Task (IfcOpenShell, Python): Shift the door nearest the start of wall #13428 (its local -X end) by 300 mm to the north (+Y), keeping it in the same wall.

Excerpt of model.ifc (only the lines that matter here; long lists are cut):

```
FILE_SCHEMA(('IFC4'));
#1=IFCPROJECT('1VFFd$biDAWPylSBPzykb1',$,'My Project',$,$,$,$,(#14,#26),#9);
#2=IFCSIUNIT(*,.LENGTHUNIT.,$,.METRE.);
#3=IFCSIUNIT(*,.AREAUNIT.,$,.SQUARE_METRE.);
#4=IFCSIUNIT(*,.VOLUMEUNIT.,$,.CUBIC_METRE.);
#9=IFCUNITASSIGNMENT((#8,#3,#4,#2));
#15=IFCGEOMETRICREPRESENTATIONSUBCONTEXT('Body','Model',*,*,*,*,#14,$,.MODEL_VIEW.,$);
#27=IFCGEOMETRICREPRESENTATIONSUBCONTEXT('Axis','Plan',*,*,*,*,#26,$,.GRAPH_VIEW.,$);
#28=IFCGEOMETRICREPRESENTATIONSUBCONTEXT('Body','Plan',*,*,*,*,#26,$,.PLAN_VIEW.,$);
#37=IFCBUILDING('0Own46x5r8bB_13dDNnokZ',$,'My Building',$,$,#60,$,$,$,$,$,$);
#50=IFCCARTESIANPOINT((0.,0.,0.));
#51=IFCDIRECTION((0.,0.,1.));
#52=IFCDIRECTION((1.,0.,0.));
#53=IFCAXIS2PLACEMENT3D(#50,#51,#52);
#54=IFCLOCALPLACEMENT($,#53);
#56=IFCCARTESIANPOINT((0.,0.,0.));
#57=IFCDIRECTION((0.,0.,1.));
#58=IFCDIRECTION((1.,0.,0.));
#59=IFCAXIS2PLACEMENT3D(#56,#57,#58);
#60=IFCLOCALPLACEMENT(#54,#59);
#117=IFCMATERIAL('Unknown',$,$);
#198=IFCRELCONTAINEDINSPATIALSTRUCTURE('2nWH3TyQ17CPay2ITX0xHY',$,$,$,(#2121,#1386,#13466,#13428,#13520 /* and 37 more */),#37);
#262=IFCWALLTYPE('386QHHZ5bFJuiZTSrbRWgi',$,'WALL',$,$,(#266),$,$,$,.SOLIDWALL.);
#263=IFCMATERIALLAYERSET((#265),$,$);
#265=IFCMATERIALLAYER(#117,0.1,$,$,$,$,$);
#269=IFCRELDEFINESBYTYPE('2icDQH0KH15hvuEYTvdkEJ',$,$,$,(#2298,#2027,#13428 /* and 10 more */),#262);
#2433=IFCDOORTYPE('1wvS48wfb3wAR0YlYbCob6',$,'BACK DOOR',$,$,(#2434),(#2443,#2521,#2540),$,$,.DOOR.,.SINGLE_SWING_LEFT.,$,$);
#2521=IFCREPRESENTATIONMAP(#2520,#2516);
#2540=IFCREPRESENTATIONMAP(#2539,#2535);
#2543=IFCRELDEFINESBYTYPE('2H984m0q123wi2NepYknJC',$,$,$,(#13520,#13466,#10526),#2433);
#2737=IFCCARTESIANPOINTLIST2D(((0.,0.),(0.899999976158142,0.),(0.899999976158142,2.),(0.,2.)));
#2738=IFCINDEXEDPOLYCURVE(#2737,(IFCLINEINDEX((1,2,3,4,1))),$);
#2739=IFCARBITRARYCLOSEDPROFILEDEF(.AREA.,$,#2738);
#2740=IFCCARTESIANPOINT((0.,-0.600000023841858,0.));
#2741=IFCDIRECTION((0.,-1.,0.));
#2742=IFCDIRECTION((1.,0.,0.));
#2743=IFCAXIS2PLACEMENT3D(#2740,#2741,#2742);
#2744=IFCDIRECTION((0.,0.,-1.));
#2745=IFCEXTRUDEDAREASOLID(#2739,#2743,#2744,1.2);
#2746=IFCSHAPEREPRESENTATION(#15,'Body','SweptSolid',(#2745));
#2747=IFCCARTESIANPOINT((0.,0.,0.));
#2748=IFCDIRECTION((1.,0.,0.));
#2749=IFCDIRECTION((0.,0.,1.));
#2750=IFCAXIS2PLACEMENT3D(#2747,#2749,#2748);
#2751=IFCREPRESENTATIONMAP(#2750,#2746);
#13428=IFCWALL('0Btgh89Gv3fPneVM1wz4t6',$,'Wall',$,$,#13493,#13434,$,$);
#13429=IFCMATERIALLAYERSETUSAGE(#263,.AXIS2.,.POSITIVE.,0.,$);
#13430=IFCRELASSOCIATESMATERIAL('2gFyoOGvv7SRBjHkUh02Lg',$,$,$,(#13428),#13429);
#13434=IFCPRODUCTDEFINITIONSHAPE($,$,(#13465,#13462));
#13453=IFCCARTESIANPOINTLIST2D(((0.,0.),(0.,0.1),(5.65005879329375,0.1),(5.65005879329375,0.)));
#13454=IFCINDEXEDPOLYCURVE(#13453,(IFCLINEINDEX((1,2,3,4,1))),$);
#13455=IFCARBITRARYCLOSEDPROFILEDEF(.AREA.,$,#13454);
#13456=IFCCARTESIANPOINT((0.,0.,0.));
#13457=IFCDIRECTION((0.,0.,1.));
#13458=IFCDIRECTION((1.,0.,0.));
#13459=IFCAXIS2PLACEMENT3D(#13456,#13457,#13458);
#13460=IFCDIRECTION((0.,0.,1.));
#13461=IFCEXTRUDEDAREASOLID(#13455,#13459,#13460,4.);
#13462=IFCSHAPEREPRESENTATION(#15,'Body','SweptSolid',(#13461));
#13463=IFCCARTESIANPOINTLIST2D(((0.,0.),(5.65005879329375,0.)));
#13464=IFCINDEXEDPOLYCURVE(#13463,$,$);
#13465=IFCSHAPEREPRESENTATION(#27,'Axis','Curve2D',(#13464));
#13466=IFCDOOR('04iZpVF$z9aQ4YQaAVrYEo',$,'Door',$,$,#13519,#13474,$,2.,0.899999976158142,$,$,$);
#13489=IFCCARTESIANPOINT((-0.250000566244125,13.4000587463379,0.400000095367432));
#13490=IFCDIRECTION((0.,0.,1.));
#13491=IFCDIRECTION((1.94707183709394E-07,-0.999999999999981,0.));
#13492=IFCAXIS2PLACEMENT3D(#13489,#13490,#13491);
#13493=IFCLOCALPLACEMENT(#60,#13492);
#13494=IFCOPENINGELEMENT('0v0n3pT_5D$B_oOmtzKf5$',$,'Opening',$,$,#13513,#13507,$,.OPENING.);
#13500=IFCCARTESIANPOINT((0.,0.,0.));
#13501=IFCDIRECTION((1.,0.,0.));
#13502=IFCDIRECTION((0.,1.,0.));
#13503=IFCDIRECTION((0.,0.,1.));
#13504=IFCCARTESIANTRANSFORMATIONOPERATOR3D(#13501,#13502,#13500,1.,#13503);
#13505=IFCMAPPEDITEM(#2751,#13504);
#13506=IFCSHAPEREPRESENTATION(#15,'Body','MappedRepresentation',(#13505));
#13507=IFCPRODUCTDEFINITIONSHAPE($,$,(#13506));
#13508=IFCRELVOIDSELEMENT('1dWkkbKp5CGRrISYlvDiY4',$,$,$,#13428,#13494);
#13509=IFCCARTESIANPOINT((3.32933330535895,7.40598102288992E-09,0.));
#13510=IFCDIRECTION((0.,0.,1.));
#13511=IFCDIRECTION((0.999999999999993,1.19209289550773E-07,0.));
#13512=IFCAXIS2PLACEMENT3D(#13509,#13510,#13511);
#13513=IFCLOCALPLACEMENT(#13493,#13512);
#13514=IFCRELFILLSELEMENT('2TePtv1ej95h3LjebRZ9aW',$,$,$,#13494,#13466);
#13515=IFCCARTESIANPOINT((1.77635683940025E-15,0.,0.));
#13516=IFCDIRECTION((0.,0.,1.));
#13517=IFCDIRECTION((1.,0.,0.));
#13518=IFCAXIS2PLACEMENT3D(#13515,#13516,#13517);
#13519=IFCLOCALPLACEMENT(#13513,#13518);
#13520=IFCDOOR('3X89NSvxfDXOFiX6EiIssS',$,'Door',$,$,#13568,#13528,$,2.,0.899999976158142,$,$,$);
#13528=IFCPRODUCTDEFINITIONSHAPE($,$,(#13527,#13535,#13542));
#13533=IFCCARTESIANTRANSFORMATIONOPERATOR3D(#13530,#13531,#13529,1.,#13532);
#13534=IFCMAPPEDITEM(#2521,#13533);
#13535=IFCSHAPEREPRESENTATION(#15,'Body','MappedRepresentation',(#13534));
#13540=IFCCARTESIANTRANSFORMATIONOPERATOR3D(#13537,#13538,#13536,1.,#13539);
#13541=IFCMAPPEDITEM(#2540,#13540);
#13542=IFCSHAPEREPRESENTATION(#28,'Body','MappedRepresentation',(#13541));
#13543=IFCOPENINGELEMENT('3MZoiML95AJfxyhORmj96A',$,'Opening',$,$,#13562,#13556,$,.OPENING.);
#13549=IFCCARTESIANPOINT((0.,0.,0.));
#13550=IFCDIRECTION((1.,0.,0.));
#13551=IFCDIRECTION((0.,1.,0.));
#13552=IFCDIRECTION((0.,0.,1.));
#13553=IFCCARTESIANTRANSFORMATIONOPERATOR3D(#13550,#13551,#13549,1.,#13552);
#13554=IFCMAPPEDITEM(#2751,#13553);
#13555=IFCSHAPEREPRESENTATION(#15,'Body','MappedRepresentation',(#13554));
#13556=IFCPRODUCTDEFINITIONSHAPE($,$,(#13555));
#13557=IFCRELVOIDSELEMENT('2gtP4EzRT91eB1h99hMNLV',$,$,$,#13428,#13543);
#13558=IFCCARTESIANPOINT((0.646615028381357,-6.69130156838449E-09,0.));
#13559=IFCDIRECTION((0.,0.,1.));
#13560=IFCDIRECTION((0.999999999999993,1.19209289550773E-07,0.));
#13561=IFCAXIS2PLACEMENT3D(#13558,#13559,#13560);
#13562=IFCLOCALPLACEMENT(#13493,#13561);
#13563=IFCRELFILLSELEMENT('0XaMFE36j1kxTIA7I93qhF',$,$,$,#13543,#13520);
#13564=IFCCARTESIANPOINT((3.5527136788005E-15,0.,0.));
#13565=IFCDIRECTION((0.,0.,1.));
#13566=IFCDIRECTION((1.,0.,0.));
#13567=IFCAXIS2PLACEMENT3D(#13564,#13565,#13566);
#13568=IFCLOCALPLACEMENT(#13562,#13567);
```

```python
import ifcopenshell
import ifcopenshell.api.geometry
import ifcopenshell.util.placement

model = ifcopenshell.open("model.ifc")

door = model.by_guid("3X89NSvxfDXOFiX6EiIssS")
opening = door.FillsVoids[0].RelatingOpeningElement
wall = opening.VoidsElements[0].RelatingBuildingElement

wall_matrix = ifcopenshell.util.placement.get_local_placement(wall.ObjectPlacement)
shift = wall_matrix[:3, 0] * -0.3
before = ifcopenshell.util.placement.get_local_placement(door.ObjectPlacement)[:3, 3].copy()

# The door is placed relative to its opening, so it follows when the opening moves.
matrix = ifcopenshell.util.placement.get_local_placement(opening.ObjectPlacement)
matrix[:3, 3] += shift
ifcopenshell.api.geometry.edit_object_placement(
    model, product=opening, matrix=matrix, is_si=False, should_transform_children=True
)

after = ifcopenshell.util.placement.get_local_placement(door.ObjectPlacement)[:3, 3]
print("door moved by", (after - before).round(3) + 0.0)

model.write("model_edited.ifc")
```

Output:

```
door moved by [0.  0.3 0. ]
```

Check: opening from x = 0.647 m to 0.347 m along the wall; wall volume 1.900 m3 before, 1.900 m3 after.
